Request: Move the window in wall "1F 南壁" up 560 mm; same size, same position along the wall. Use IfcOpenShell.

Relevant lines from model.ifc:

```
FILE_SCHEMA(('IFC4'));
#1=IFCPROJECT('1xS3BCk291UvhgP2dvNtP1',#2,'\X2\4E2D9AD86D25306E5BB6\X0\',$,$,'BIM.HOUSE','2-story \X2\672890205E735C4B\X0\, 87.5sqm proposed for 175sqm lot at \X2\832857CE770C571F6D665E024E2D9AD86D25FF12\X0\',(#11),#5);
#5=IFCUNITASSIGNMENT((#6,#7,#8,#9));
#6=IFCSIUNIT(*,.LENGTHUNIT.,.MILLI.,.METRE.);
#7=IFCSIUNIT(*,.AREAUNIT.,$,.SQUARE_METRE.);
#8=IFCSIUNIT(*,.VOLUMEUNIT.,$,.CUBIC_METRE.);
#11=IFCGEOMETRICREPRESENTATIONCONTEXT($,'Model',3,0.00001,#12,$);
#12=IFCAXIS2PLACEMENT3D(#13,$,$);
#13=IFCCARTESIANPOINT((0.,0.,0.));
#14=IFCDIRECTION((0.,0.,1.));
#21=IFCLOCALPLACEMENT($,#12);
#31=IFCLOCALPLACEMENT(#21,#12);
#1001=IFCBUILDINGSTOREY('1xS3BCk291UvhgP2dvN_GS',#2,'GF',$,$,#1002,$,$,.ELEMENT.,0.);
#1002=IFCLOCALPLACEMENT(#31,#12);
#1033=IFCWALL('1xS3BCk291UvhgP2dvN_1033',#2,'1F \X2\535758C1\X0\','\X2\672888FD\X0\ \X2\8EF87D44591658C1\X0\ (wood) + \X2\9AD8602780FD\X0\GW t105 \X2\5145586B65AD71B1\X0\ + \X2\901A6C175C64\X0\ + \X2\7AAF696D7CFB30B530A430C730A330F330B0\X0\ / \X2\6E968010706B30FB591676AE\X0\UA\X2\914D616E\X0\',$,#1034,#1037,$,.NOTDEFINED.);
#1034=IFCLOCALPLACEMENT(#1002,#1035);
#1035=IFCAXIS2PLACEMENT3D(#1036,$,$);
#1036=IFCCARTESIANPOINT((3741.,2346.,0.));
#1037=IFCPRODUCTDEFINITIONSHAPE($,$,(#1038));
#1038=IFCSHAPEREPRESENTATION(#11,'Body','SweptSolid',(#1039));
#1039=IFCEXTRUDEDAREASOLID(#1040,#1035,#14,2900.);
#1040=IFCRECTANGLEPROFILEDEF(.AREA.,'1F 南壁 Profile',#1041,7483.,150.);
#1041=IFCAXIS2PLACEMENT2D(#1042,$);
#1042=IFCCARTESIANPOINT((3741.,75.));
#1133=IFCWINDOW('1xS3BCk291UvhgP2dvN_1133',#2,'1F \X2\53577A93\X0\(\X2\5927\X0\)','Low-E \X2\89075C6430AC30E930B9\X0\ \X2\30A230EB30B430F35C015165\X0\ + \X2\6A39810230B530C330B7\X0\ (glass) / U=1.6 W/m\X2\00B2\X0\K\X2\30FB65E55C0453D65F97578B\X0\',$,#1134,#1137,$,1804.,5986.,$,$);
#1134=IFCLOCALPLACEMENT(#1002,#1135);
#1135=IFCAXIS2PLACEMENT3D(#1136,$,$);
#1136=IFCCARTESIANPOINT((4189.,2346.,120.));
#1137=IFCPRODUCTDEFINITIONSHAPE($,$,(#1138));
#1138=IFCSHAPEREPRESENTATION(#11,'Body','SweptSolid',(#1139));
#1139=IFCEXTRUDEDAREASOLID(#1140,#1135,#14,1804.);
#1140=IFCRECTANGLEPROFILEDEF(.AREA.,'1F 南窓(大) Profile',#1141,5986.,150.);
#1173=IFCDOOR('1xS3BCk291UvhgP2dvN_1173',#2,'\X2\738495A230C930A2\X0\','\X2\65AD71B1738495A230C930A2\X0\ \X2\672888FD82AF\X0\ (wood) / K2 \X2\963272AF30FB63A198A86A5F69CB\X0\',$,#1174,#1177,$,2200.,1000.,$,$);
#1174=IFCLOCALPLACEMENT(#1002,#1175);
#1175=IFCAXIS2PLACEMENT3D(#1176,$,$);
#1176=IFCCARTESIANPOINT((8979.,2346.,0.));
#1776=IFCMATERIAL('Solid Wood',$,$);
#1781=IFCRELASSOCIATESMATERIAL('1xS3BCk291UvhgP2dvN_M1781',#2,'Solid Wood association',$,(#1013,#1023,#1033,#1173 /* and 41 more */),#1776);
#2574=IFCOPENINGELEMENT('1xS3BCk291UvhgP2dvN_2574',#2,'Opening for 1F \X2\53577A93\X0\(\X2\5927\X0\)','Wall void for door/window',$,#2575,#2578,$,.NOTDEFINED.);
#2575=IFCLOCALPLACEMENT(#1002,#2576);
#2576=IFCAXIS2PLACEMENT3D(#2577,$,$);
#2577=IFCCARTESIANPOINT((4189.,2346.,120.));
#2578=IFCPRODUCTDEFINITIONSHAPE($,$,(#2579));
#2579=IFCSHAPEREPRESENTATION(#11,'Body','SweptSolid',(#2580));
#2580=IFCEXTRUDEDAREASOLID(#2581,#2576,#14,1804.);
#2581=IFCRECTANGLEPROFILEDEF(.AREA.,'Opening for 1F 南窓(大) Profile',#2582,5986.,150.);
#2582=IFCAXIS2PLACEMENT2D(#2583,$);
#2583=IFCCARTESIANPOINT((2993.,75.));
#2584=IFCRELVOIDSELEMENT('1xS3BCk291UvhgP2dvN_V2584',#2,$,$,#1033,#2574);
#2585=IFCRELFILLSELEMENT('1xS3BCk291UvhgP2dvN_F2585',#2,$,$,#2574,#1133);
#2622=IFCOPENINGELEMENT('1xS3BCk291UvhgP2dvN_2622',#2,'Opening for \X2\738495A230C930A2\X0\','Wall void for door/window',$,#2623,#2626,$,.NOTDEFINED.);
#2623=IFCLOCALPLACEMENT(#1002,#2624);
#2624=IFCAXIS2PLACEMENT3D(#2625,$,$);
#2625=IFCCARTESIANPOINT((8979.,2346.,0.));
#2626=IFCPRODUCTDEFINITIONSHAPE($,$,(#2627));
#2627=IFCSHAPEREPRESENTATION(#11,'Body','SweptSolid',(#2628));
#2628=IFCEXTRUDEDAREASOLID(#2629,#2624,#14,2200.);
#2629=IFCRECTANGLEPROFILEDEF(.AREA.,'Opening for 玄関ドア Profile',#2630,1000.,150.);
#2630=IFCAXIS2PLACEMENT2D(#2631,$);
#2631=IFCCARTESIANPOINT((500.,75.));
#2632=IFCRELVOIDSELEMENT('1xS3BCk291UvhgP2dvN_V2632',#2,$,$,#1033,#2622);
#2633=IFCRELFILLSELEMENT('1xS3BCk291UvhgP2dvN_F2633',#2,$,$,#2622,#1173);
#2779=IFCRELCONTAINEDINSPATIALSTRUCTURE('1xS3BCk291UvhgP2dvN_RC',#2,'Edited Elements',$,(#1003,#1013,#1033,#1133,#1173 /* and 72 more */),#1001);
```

```python
import numpy as np
import ifcopenshell
import ifcopenshell.api.geometry
import ifcopenshell.util.placement
import ifcopenshell.util.unit

model = ifcopenshell.open("model.ifc")
unit_scale = ifcopenshell.util.unit.calculate_unit_scale(model)

window = model.by_guid("1xS3BCk291UvhgP2dvN_1133")
opening = window.FillsVoids[0].RelatingOpeningElement
dz = 560.0

shift = np.array([0.0, 0.0, dz])
# The window is not placed relative to its opening, so move both.
for product in (opening, window):
    matrix = ifcopenshell.util.placement.get_local_placement(product.ObjectPlacement)
    matrix[:3, 3] += shift
    ifcopenshell.api.geometry.edit_object_placement(model, product=product, matrix=matrix, is_si=False)

print(f"moved by {dz * unit_scale:+.3f} m")

model.write("model-out.ifc")
```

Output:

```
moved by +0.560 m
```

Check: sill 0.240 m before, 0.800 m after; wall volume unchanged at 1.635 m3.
